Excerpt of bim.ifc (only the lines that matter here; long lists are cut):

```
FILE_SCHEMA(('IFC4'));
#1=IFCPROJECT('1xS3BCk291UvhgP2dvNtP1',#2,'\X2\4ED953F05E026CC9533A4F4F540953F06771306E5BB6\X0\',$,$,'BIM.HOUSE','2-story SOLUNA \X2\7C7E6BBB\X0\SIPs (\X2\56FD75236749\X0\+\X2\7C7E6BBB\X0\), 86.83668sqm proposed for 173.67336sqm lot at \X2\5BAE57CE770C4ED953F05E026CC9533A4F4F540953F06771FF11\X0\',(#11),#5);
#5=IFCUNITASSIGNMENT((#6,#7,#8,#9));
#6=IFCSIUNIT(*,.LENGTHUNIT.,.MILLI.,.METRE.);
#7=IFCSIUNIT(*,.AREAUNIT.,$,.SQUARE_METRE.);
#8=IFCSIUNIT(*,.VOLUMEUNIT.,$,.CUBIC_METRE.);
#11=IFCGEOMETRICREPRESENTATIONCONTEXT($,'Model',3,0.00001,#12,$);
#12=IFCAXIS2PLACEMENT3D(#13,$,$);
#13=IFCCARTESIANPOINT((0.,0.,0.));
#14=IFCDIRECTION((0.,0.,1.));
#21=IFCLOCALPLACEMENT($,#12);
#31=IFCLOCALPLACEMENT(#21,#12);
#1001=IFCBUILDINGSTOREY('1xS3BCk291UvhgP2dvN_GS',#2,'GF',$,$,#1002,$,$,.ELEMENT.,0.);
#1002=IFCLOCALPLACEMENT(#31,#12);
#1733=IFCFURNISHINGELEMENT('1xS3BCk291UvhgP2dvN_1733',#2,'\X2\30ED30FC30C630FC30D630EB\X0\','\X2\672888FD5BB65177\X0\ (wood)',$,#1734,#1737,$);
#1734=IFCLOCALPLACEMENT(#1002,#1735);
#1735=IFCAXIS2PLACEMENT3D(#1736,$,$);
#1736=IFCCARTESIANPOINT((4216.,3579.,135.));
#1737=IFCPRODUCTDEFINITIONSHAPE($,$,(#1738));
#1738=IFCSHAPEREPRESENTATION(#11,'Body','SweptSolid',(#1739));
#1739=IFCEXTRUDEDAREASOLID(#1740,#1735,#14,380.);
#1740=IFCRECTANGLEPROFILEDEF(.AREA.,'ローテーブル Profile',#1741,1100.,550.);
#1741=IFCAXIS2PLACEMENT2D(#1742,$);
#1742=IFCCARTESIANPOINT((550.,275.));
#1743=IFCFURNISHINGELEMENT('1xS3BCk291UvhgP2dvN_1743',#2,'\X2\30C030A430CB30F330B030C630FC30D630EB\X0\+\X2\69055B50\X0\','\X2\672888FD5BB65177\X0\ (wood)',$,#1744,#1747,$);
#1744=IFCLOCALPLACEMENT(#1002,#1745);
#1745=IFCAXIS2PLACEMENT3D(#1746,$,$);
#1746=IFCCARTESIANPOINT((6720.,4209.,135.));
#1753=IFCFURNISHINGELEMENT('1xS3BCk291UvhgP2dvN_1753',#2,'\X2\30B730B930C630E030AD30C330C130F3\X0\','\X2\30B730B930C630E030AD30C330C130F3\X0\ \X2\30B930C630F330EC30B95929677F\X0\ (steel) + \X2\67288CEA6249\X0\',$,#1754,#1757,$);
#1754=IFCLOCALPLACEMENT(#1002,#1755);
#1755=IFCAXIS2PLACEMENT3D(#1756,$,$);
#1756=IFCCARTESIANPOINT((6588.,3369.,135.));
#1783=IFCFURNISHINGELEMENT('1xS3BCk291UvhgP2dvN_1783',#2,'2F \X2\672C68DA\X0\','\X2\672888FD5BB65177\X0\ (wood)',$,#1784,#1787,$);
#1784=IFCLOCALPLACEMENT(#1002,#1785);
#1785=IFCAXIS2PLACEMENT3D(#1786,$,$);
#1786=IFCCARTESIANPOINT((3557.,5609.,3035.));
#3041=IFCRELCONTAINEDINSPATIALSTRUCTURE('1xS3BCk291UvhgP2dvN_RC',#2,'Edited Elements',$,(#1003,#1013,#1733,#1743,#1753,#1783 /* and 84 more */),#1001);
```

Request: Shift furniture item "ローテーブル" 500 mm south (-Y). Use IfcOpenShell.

```python
import ifcopenshell
import ifcopenshell.api.geometry
import ifcopenshell.util.placement

model = ifcopenshell.open("bim.ifc")

item = model.by_guid("1xS3BCk291UvhgP2dvN_1733")
matrix = ifcopenshell.util.placement.get_local_placement(item.ObjectPlacement)
matrix[1, 3] -= 500.0
ifcopenshell.api.geometry.edit_object_placement(model, product=item, matrix=matrix, is_si=False)

print(ifcopenshell.util.placement.get_local_placement(item.ObjectPlacement).round(3) + 0.0)

model.write("bim_v2.ifc")
```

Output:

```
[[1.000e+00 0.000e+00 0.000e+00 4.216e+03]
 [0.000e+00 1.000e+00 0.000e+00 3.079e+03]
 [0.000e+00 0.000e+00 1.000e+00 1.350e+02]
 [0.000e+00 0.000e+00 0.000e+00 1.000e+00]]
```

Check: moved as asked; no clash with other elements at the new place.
